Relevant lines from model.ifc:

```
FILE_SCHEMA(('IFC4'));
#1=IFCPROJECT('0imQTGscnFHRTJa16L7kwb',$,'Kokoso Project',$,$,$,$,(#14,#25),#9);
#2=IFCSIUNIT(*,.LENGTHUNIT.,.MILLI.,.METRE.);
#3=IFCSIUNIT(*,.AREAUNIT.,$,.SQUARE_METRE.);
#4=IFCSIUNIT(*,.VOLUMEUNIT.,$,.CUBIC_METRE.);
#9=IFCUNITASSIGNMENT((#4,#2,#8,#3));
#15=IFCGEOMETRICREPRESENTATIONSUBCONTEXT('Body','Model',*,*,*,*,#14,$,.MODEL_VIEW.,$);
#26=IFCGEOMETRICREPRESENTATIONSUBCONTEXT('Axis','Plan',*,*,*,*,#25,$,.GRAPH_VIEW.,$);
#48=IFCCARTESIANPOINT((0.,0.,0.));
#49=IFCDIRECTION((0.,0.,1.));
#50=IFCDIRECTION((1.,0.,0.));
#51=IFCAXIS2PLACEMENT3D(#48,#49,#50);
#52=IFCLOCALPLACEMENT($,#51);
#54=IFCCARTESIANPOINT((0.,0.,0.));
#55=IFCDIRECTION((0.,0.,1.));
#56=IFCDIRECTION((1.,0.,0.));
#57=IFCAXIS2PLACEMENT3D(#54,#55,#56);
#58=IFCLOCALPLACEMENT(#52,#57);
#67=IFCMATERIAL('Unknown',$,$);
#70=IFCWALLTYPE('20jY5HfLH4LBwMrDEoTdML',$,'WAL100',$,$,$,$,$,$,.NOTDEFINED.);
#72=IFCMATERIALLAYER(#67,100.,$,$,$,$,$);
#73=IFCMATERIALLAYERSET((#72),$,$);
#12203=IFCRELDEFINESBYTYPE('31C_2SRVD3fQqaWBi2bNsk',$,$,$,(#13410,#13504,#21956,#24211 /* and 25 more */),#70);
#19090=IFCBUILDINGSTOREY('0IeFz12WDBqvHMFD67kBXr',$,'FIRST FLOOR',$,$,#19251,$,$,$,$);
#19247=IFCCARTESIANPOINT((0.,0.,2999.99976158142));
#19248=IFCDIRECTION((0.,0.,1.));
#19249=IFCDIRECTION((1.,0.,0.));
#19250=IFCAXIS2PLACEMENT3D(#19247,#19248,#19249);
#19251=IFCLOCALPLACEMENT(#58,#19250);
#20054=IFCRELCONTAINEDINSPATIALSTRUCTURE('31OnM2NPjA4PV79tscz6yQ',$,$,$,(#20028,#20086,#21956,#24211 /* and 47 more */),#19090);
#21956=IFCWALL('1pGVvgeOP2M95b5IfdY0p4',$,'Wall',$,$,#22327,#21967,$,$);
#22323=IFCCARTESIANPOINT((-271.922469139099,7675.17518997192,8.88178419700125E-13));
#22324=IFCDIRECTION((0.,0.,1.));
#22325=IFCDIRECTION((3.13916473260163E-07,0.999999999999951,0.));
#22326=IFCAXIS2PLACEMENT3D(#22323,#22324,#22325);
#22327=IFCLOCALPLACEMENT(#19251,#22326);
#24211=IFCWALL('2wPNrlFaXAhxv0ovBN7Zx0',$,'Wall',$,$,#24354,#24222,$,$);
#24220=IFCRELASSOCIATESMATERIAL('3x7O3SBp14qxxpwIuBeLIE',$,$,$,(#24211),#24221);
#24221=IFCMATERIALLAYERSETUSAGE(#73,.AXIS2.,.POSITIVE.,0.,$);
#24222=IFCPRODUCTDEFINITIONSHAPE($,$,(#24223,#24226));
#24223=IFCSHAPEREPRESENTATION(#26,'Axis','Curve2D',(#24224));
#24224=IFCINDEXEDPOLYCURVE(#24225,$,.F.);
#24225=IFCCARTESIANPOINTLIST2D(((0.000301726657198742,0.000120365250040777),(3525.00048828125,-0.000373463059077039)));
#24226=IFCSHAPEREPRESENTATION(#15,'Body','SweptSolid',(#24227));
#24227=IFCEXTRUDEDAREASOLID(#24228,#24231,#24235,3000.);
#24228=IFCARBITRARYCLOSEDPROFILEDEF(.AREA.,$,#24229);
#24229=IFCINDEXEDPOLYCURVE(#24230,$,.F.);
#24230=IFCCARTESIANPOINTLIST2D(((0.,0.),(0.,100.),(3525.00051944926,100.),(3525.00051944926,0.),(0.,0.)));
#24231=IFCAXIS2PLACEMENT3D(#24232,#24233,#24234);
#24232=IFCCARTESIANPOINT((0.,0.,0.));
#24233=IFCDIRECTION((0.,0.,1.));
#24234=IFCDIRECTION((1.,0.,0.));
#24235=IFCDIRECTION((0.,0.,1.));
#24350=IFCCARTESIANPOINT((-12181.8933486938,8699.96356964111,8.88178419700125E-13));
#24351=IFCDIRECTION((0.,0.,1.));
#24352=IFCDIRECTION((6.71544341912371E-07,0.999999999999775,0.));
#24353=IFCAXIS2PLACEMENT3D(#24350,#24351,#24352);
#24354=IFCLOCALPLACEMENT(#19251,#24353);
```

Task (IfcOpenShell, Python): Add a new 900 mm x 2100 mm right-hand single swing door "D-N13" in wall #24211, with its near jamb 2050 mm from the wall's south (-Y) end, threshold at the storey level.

```python
import numpy as np
import ifcopenshell
import ifcopenshell.api.feature
import ifcopenshell.api.geometry
import ifcopenshell.api.root
import ifcopenshell.api.spatial
import ifcopenshell.geom
import ifcopenshell.util.element
import ifcopenshell.util.placement
import ifcopenshell.util.representation
import ifcopenshell.util.shape
import ifcopenshell.util.unit

model = ifcopenshell.open("model.ifc")
unit_scale = ifcopenshell.util.unit.calculate_unit_scale(model)
settings = ifcopenshell.geom.settings()


def volume(element):
    """Net volume in cubic metres, openings subtracted."""
    shape = ifcopenshell.geom.create_shape(settings, element)
    return ifcopenshell.util.shape.get_volume(shape.geometry)


wall = model.by_guid("2wPNrlFaXAhxv0ovBN7Zx0")
storey = ifcopenshell.util.element.get_container(wall, ifc_class="IfcBuildingStorey")
context = ifcopenshell.util.representation.get_context(model, "Model", "Body", "MODEL_VIEW")
before = volume(wall)

width, height, from_end, sill = 0.9, 2.1, 2.05, 0.0  # metres

# The wall runs along its own X axis, and the end named is its -X end.
wall_shape = ifcopenshell.geom.create_shape(settings, wall)
x, y, z = ifcopenshell.util.shape.get_vertices(wall_shape.geometry).T
start = x.min() + from_end
face, thickness = float(y.min()), float(y.max() - y.min())
wall_matrix = ifcopenshell.util.placement.get_local_placement(wall.ObjectPlacement)
level = ifcopenshell.util.placement.get_local_placement(storey.ObjectPlacement)[2, 3]


def in_wall(x, y):
    """Placement at x, y metres in the wall's axes, at sill height."""
    matrix = wall_matrix.copy()
    matrix[:, 3] = wall_matrix @ np.array([x / unit_scale, y / unit_scale, 0.0, 1.0])
    matrix[2, 3] = level + sill / unit_scale
    return matrix


# Opening: a box that overshoots both wall faces by 50 mm.
opening = ifcopenshell.api.root.create_entity(model, ifc_class="IfcOpeningElement", predefined_type="OPENING")
box = ifcopenshell.api.geometry.add_wall_representation(
    model, context=context, length=width, height=height, thickness=thickness + 0.1
)
ifcopenshell.api.geometry.assign_representation(model, product=opening, representation=box)
ifcopenshell.api.geometry.edit_object_placement(model, product=opening, matrix=in_wall(start, face - 0.05), is_si=False)
ifcopenshell.api.feature.add_feature(model, feature=opening, element=wall)

door = ifcopenshell.api.root.create_entity(model, ifc_class="IfcDoor", name="D-N13", predefined_type="DOOR")
door.OverallWidth, door.OverallHeight = width / unit_scale, height / unit_scale
door.OperationType = "SINGLE_SWING_RIGHT"
body = ifcopenshell.api.geometry.add_door_representation(
    model,
    context=context,
    overall_width=door.OverallWidth,
    overall_height=door.OverallHeight,
    operation_type="SINGLE_SWING_RIGHT",
    lining_properties={"LiningDepth": thickness / unit_scale, "ThresholdDepth": thickness / unit_scale},
)
ifcopenshell.api.geometry.assign_representation(model, product=door, representation=body)
ifcopenshell.api.spatial.assign_container(model, products=[door], relating_structure=storey)
ifcopenshell.api.feature.add_filling(model, opening=opening, element=door)

# The lining spans the wall, so the door starts at the wall face.
ifcopenshell.api.geometry.edit_object_placement(model, product=door, matrix=in_wall(start, face), is_si=False)

after = volume(wall)

print(f"wall volume {before:.3f} -> {after:.3f} m3")

model.write("model_v2.ifc")
```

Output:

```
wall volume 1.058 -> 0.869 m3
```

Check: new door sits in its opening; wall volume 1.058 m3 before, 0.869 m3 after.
